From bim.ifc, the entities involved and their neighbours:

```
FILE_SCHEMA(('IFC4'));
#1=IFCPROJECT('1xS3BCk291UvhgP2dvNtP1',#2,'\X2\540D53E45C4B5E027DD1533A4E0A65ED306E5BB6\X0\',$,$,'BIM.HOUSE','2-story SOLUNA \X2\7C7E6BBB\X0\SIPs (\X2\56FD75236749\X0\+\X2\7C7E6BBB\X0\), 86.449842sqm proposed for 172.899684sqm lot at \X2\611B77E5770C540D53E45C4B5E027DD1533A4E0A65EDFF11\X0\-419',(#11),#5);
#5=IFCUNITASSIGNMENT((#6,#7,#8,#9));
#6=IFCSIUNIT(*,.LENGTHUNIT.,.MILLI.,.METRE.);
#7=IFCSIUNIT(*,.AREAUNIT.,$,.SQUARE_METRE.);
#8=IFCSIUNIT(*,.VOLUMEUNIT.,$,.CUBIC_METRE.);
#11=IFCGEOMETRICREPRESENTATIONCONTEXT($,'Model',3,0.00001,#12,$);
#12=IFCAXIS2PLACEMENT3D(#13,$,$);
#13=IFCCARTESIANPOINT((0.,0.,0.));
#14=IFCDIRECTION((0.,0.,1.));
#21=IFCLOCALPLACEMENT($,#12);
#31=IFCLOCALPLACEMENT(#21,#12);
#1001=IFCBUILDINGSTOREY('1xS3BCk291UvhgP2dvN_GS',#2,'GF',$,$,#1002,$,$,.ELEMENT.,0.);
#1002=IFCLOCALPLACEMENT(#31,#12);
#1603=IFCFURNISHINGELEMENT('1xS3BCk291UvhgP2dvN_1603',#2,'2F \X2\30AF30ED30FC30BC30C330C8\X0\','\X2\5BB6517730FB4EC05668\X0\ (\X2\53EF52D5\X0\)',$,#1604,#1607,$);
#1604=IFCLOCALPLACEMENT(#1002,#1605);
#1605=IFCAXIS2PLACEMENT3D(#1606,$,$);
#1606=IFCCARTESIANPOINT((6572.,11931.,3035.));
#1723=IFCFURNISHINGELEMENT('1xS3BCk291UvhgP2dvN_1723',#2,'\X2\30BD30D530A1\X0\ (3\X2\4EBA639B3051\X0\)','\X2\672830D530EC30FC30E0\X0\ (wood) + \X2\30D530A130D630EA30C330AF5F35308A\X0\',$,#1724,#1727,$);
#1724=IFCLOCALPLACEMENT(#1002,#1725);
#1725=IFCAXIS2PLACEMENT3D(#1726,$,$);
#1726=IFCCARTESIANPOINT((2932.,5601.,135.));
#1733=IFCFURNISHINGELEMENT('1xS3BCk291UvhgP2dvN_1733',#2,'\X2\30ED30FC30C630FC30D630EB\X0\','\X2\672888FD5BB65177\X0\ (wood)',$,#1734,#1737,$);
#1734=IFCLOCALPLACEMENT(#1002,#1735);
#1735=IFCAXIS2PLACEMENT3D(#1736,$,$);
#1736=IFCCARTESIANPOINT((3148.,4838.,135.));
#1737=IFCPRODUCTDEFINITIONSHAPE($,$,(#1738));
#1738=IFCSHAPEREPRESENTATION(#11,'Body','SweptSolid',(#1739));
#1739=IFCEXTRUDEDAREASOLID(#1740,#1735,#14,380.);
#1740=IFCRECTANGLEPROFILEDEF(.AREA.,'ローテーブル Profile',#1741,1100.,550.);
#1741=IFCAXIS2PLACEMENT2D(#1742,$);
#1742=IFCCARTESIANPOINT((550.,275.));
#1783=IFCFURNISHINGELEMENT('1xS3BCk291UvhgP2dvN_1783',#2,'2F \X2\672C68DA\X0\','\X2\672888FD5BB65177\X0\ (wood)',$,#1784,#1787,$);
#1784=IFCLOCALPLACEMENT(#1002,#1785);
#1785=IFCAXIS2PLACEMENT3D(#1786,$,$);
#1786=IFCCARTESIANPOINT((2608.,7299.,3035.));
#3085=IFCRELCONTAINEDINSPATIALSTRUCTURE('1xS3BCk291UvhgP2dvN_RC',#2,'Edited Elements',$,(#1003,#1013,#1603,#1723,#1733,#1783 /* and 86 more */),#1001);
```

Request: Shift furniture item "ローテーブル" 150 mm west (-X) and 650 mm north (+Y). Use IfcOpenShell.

```python
import ifcopenshell
import ifcopenshell.api.geometry
import ifcopenshell.util.placement
import ifcopenshell.util.unit

model = ifcopenshell.open("bim.ifc")
unit_scale = ifcopenshell.util.unit.calculate_unit_scale(model)

item = model.by_guid("1xS3BCk291UvhgP2dvN_1733")
matrix = ifcopenshell.util.placement.get_local_placement(item.ObjectPlacement)
matrix[0, 3] -= 0.15 / unit_scale
matrix[1, 3] += 0.65 / unit_scale
ifcopenshell.api.geometry.edit_object_placement(model, product=item, matrix=matrix, is_si=False)

print(ifcopenshell.util.placement.get_local_placement(item.ObjectPlacement).round(3) + 0.0)

model.write("bim-out.ifc")
```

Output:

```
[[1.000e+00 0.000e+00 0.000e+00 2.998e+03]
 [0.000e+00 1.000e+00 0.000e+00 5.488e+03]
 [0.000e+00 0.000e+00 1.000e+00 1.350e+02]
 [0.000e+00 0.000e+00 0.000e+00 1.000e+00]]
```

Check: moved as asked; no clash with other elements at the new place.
